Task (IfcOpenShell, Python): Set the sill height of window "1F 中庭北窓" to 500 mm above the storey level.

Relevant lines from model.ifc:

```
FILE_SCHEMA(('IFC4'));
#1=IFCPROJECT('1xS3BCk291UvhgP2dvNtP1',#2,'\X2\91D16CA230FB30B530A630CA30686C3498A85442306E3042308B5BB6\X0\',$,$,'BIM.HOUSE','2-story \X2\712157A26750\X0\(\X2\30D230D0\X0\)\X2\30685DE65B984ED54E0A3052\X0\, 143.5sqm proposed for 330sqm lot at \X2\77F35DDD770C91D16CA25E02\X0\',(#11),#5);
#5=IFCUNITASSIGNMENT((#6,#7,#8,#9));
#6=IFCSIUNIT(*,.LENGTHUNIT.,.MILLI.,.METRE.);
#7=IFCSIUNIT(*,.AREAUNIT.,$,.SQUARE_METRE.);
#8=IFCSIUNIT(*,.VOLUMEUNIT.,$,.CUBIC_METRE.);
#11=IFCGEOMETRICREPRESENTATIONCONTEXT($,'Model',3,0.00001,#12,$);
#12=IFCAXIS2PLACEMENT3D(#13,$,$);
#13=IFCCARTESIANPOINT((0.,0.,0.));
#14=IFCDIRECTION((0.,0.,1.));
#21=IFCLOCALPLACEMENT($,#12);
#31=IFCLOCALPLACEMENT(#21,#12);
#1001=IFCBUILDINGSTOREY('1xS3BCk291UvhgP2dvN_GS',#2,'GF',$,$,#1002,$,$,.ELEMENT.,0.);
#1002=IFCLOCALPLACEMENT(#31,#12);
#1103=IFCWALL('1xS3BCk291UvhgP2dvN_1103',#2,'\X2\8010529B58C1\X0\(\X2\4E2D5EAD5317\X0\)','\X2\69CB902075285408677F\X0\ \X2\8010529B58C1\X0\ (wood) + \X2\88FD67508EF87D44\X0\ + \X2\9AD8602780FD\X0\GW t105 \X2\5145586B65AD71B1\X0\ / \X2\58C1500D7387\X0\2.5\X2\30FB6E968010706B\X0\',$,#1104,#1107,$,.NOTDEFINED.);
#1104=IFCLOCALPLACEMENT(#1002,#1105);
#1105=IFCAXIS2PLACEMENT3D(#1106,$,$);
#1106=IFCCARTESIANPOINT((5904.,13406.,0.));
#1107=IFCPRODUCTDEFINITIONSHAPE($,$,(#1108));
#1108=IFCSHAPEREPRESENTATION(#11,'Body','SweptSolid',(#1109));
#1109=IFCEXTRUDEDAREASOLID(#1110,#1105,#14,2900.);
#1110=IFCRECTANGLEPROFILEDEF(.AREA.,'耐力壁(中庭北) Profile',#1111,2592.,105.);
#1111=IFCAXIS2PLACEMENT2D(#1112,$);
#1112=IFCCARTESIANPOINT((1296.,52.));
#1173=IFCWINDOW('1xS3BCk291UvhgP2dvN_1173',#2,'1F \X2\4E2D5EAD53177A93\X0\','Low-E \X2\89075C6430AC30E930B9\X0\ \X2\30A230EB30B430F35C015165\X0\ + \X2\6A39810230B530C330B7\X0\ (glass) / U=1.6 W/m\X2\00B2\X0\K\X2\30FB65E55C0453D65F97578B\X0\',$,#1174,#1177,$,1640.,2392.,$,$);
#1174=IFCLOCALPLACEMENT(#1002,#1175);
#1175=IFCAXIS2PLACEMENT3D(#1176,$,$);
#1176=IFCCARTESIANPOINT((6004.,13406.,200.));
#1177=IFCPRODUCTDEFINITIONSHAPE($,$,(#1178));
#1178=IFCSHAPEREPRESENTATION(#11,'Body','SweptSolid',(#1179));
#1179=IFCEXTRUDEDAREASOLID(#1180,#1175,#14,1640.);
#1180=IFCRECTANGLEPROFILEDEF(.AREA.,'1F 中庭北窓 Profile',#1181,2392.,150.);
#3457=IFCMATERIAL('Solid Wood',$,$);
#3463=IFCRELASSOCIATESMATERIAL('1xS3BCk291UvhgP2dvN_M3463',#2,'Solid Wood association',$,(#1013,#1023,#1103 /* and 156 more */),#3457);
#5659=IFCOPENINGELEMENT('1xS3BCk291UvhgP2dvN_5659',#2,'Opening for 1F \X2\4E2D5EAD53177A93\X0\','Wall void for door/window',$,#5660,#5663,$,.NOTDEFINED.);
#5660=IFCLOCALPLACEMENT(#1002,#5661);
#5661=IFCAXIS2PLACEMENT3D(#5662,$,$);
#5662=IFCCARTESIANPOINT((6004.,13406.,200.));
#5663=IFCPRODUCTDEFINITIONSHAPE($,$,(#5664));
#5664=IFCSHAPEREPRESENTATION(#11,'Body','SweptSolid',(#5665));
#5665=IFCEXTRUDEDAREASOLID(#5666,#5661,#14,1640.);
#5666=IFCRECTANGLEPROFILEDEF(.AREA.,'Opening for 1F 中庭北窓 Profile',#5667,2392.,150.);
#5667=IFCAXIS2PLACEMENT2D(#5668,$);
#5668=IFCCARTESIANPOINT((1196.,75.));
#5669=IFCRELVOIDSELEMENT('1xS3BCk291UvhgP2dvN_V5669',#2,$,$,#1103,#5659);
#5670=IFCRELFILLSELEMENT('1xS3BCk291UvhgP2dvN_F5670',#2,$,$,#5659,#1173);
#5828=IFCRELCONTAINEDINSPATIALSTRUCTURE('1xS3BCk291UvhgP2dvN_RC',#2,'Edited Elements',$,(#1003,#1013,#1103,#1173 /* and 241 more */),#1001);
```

```python
import numpy as np
import ifcopenshell
import ifcopenshell.api.geometry
import ifcopenshell.geom
import ifcopenshell.util.element
import ifcopenshell.util.placement
import ifcopenshell.util.shape
import ifcopenshell.util.unit

model = ifcopenshell.open("model.ifc")
unit_scale = ifcopenshell.util.unit.calculate_unit_scale(model)

window = model.by_guid("1xS3BCk291UvhgP2dvN_1173")
opening = window.FillsVoids[0].RelatingOpeningElement
storey = ifcopenshell.util.element.get_container(window, ifc_class="IfcBuildingStorey")
level = ifcopenshell.util.placement.get_local_placement(storey.ObjectPlacement)[2, 3]

# The opening's origin need not be at the sill, so measure its lowest point.
shape = ifcopenshell.geom.create_shape(ifcopenshell.geom.settings(), opening)
bottom = ifcopenshell.util.shape.get_shape_bottom_elevation(shape, shape.geometry) / unit_scale
dz = level + 0.5 / unit_scale - bottom

shift = np.array([0.0, 0.0, dz])
# The window is not placed relative to its opening, so move both.
for product in (opening, window):
    matrix = ifcopenshell.util.placement.get_local_placement(product.ObjectPlacement)
    matrix[:3, 3] += shift
    ifcopenshell.api.geometry.edit_object_placement(model, product=product, matrix=matrix, is_si=False)

print(f"moved by {dz * unit_scale:+.3f} m")

model.write("model_v2.ifc")
```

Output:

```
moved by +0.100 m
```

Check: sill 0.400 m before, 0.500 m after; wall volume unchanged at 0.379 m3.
